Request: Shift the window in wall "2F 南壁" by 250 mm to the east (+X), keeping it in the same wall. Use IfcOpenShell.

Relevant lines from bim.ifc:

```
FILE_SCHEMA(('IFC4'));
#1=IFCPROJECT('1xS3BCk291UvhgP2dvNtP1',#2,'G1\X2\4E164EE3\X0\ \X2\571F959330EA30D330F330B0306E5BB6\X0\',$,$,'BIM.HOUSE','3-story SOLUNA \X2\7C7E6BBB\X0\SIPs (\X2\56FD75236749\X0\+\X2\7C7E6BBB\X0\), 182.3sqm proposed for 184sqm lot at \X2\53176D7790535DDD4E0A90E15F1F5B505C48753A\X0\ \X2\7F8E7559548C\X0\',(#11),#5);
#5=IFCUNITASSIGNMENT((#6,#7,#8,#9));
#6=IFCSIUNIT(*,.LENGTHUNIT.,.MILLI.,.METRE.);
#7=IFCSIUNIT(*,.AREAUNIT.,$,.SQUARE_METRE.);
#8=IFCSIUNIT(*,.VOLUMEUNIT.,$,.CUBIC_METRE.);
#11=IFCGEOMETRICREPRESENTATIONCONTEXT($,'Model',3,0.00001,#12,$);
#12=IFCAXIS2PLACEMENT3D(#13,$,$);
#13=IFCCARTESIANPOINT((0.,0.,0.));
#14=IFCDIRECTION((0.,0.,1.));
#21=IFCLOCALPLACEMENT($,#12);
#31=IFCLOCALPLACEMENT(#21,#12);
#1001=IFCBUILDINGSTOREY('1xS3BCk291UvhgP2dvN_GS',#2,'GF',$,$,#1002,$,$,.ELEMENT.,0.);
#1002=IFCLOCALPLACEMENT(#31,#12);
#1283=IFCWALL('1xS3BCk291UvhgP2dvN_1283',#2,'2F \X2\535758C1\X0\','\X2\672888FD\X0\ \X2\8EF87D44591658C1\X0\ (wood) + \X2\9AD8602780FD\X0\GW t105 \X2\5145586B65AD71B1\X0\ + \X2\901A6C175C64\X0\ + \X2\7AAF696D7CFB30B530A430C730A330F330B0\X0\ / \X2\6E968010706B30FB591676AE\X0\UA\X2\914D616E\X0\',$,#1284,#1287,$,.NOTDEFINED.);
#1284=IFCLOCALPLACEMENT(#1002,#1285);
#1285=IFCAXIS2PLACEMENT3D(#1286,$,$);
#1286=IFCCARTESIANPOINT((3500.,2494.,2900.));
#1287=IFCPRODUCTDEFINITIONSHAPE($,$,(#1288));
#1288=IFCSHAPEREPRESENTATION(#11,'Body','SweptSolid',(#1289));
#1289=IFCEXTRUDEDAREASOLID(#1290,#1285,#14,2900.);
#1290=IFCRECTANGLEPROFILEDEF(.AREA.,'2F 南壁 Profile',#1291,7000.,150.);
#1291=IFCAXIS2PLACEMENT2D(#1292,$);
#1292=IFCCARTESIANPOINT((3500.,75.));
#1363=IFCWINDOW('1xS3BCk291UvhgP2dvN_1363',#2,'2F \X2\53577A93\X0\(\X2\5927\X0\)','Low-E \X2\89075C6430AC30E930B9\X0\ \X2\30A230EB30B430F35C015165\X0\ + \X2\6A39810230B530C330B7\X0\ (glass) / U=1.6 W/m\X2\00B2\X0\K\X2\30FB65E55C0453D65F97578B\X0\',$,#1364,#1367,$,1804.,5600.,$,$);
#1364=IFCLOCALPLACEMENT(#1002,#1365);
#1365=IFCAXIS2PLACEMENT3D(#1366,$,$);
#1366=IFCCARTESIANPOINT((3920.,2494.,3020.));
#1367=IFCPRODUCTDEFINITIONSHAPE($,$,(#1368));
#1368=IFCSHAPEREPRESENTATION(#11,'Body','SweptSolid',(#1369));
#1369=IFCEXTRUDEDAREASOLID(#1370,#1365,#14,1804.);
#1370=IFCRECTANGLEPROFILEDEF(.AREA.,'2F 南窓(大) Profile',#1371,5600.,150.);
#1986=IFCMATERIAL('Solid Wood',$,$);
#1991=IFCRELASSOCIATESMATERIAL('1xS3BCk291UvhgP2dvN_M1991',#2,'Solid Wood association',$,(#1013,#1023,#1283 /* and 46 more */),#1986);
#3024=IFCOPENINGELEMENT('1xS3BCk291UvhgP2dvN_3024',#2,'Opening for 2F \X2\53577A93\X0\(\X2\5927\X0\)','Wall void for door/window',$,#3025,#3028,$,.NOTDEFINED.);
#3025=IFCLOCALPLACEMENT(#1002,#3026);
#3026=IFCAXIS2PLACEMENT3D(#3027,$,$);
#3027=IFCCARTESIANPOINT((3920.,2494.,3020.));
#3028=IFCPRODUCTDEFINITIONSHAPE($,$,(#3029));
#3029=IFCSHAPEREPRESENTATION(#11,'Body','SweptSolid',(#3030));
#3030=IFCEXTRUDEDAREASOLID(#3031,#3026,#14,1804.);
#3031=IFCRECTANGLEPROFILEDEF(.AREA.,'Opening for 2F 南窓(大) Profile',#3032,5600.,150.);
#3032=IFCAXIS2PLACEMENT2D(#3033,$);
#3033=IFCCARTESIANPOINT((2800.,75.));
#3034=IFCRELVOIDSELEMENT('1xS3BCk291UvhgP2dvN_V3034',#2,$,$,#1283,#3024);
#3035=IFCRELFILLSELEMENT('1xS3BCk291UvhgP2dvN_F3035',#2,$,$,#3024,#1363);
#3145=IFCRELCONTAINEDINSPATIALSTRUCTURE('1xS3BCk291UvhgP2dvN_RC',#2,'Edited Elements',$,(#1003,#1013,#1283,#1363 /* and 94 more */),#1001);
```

```python
import ifcopenshell
import ifcopenshell.api.geometry
import ifcopenshell.util.placement

model = ifcopenshell.open("bim.ifc")

window = model.by_id(1363)
opening = window.FillsVoids[0].RelatingOpeningElement
wall = opening.VoidsElements[0].RelatingBuildingElement

wall_matrix = ifcopenshell.util.placement.get_local_placement(wall.ObjectPlacement)
shift = wall_matrix[:3, 0] * 250.0
before = ifcopenshell.util.placement.get_local_placement(window.ObjectPlacement)[:3, 3].copy()

# The window is not placed relative to its opening, so move both.
for product in (opening, window):
    matrix = ifcopenshell.util.placement.get_local_placement(product.ObjectPlacement)
    matrix[:3, 3] += shift
    ifcopenshell.api.geometry.edit_object_placement(model, product=product, matrix=matrix, is_si=False)

after = ifcopenshell.util.placement.get_local_placement(window.ObjectPlacement)[:3, 3]
print("window moved by", (after - before).round(3) + 0.0)

model.write("bim_updated.ifc")
```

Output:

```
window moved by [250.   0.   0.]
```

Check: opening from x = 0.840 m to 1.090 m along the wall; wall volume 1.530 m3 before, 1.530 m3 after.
